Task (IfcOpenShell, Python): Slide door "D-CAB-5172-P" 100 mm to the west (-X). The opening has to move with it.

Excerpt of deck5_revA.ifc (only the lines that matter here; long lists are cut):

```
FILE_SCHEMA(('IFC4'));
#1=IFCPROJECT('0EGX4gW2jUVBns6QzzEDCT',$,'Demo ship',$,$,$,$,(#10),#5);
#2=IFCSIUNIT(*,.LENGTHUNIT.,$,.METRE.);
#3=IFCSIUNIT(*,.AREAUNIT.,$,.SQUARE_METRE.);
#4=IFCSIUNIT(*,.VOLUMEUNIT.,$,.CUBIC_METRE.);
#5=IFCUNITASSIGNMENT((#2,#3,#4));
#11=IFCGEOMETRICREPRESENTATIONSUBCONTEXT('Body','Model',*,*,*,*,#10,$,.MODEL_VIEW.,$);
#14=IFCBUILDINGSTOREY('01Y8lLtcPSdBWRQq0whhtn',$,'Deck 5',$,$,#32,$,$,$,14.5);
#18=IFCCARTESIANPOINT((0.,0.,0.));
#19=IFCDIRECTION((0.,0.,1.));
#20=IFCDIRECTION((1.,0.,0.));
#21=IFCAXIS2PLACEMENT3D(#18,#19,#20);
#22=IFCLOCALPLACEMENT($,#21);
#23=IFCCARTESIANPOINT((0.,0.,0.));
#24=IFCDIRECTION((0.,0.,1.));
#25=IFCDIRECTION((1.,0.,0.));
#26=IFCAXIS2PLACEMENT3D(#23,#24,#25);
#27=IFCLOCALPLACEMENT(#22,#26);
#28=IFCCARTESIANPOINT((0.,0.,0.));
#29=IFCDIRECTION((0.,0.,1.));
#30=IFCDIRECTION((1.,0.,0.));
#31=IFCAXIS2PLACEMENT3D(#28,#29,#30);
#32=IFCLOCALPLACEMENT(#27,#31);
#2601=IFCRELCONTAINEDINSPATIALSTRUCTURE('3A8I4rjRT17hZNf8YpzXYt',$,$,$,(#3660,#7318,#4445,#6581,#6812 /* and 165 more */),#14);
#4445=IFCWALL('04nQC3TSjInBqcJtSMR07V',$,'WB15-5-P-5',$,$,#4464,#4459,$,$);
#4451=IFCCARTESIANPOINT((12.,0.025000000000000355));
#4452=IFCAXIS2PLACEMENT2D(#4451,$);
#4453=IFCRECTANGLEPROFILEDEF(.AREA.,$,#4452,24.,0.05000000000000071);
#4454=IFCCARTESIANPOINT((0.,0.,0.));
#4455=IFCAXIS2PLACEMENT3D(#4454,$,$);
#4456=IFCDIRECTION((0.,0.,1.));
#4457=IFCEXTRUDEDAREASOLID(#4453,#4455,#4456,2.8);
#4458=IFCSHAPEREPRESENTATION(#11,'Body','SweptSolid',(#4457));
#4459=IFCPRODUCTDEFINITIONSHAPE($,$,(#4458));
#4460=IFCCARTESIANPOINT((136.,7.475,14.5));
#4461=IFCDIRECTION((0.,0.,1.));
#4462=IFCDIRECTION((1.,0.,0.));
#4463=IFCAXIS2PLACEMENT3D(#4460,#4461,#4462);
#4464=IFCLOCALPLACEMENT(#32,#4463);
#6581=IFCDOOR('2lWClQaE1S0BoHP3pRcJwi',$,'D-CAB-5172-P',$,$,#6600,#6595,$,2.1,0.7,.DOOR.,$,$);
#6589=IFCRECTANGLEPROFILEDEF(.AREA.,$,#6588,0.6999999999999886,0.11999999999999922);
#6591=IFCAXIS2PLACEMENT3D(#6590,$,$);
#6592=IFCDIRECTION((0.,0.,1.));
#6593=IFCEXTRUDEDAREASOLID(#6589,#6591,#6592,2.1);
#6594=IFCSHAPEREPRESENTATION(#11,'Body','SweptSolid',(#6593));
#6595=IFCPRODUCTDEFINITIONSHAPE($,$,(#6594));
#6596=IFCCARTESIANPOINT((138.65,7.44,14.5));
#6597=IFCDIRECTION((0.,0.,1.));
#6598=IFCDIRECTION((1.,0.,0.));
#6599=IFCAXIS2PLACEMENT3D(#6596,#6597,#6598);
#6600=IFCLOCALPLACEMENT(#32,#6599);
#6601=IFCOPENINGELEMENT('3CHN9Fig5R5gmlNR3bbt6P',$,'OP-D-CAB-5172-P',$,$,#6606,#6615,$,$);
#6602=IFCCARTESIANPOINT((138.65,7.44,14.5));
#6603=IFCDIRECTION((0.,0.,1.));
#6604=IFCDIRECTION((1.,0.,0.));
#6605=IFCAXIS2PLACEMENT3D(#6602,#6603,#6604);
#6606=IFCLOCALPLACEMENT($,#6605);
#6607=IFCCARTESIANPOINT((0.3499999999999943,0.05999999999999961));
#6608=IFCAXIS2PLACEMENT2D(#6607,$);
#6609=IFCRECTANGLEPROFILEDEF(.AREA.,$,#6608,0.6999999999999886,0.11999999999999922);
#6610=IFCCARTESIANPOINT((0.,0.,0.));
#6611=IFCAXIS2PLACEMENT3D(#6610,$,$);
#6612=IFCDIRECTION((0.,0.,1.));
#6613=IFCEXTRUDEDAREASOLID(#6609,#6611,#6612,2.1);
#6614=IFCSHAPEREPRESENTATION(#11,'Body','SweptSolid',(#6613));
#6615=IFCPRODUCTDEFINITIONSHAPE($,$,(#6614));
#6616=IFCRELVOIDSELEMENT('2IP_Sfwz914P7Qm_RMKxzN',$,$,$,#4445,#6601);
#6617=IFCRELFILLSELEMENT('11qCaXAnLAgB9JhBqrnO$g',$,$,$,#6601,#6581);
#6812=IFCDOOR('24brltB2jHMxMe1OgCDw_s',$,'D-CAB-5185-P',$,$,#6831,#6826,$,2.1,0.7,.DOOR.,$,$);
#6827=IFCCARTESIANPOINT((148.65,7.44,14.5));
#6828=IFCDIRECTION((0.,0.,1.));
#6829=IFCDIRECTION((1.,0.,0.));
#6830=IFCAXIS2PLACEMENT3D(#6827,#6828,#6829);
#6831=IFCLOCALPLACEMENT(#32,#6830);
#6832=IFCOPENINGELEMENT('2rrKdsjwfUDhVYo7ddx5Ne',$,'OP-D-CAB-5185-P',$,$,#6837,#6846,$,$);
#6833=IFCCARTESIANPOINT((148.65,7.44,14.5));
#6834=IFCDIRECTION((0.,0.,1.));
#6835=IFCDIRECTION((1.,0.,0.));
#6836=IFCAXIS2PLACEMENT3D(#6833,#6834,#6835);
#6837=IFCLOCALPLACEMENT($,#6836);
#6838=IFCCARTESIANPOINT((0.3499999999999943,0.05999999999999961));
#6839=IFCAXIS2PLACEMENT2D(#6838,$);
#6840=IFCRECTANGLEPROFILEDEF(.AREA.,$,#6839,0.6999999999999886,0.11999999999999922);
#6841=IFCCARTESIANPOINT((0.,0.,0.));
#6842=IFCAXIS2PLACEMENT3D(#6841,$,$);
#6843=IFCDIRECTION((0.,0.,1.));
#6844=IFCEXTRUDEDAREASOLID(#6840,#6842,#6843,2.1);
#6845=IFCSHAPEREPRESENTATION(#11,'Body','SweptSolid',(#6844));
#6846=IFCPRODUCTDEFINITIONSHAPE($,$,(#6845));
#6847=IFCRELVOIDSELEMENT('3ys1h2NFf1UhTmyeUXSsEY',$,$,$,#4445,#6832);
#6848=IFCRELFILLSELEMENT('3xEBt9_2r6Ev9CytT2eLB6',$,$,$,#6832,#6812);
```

```python
import ifcopenshell
import ifcopenshell.api.geometry
import ifcopenshell.util.placement
import ifcopenshell.util.unit

model = ifcopenshell.open("deck5_revA.ifc")
unit_scale = ifcopenshell.util.unit.calculate_unit_scale(model)

door = model.by_guid("2lWClQaE1S0BoHP3pRcJwi")
opening = door.FillsVoids[0].RelatingOpeningElement
wall = opening.VoidsElements[0].RelatingBuildingElement

wall_matrix = ifcopenshell.util.placement.get_local_placement(wall.ObjectPlacement)
shift = wall_matrix[:3, 0] * -0.1 / unit_scale
before = ifcopenshell.util.placement.get_local_placement(door.ObjectPlacement)[:3, 3].copy()

# The door is not placed relative to its opening, so move both.
for product in (opening, door):
    matrix = ifcopenshell.util.placement.get_local_placement(product.ObjectPlacement)
    matrix[:3, 3] += shift
    ifcopenshell.api.geometry.edit_object_placement(model, product=product, matrix=matrix, is_si=False)

after = ifcopenshell.util.placement.get_local_placement(door.ObjectPlacement)[:3, 3]
print("door moved by", (after - before).round(3) + 0.0)

model.write("deck5_revA_rev.ifc")
```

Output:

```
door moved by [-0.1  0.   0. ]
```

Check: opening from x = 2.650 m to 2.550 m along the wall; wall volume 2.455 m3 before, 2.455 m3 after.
